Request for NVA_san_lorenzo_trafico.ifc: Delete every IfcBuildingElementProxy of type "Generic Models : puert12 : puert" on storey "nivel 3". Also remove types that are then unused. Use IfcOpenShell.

First a look at what the model holds.

```python
import ifcopenshell
import ifcopenshell.util.element

model = ifcopenshell.open("NVA_san_lorenzo_trafico.ifc")
print(model.schema)
storey = next(s for s in model.by_type("IfcBuildingStorey") if s.Name == "nivel 3")
proxies = [e for e in ifcopenshell.util.element.get_decomposition(storey) if e.is_a("IfcBuildingElementProxy")]
seen = {}
for e in proxies:
    element_type = ifcopenshell.util.element.get_type(e)
    name = element_type.Name if element_type not in (None, e) else None
    seen[name] = seen.get(name, 0) + 1
for name, count in sorted(seen.items(), key=str):
    print(count, "x", name)
```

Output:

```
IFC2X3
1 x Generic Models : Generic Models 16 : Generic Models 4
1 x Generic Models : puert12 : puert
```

```python
import ifcopenshell
import ifcopenshell.api.root
import ifcopenshell.util.element

model = ifcopenshell.open("NVA_san_lorenzo_trafico.ifc")

storey = next(s for s in model.by_type("IfcBuildingStorey") if s.Name == "nivel 3")
proxies = [e for e in ifcopenshell.util.element.get_decomposition(storey) if e.is_a("IfcBuildingElementProxy")]
targets = [e for e in proxies if (t := ifcopenshell.util.element.get_type(e)) not in (None, e) and t.Name == "Generic Models : puert12 : puert"]
types = {ifcopenshell.util.element.get_type(e) for e in targets} - {None, *targets}

for e in targets:
    ifcopenshell.api.root.remove_product(model, product=e)
print(len(targets), "removed")

unused = [t for t in types if not ifcopenshell.util.element.get_types(t)]
for t in unused:
    ifcopenshell.api.root.remove_product(model, product=t)
print(len(unused), "unused types removed")

model.write("NVA_san_lorenzo_trafico_v2.ifc")
```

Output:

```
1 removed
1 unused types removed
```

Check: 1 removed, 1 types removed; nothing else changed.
